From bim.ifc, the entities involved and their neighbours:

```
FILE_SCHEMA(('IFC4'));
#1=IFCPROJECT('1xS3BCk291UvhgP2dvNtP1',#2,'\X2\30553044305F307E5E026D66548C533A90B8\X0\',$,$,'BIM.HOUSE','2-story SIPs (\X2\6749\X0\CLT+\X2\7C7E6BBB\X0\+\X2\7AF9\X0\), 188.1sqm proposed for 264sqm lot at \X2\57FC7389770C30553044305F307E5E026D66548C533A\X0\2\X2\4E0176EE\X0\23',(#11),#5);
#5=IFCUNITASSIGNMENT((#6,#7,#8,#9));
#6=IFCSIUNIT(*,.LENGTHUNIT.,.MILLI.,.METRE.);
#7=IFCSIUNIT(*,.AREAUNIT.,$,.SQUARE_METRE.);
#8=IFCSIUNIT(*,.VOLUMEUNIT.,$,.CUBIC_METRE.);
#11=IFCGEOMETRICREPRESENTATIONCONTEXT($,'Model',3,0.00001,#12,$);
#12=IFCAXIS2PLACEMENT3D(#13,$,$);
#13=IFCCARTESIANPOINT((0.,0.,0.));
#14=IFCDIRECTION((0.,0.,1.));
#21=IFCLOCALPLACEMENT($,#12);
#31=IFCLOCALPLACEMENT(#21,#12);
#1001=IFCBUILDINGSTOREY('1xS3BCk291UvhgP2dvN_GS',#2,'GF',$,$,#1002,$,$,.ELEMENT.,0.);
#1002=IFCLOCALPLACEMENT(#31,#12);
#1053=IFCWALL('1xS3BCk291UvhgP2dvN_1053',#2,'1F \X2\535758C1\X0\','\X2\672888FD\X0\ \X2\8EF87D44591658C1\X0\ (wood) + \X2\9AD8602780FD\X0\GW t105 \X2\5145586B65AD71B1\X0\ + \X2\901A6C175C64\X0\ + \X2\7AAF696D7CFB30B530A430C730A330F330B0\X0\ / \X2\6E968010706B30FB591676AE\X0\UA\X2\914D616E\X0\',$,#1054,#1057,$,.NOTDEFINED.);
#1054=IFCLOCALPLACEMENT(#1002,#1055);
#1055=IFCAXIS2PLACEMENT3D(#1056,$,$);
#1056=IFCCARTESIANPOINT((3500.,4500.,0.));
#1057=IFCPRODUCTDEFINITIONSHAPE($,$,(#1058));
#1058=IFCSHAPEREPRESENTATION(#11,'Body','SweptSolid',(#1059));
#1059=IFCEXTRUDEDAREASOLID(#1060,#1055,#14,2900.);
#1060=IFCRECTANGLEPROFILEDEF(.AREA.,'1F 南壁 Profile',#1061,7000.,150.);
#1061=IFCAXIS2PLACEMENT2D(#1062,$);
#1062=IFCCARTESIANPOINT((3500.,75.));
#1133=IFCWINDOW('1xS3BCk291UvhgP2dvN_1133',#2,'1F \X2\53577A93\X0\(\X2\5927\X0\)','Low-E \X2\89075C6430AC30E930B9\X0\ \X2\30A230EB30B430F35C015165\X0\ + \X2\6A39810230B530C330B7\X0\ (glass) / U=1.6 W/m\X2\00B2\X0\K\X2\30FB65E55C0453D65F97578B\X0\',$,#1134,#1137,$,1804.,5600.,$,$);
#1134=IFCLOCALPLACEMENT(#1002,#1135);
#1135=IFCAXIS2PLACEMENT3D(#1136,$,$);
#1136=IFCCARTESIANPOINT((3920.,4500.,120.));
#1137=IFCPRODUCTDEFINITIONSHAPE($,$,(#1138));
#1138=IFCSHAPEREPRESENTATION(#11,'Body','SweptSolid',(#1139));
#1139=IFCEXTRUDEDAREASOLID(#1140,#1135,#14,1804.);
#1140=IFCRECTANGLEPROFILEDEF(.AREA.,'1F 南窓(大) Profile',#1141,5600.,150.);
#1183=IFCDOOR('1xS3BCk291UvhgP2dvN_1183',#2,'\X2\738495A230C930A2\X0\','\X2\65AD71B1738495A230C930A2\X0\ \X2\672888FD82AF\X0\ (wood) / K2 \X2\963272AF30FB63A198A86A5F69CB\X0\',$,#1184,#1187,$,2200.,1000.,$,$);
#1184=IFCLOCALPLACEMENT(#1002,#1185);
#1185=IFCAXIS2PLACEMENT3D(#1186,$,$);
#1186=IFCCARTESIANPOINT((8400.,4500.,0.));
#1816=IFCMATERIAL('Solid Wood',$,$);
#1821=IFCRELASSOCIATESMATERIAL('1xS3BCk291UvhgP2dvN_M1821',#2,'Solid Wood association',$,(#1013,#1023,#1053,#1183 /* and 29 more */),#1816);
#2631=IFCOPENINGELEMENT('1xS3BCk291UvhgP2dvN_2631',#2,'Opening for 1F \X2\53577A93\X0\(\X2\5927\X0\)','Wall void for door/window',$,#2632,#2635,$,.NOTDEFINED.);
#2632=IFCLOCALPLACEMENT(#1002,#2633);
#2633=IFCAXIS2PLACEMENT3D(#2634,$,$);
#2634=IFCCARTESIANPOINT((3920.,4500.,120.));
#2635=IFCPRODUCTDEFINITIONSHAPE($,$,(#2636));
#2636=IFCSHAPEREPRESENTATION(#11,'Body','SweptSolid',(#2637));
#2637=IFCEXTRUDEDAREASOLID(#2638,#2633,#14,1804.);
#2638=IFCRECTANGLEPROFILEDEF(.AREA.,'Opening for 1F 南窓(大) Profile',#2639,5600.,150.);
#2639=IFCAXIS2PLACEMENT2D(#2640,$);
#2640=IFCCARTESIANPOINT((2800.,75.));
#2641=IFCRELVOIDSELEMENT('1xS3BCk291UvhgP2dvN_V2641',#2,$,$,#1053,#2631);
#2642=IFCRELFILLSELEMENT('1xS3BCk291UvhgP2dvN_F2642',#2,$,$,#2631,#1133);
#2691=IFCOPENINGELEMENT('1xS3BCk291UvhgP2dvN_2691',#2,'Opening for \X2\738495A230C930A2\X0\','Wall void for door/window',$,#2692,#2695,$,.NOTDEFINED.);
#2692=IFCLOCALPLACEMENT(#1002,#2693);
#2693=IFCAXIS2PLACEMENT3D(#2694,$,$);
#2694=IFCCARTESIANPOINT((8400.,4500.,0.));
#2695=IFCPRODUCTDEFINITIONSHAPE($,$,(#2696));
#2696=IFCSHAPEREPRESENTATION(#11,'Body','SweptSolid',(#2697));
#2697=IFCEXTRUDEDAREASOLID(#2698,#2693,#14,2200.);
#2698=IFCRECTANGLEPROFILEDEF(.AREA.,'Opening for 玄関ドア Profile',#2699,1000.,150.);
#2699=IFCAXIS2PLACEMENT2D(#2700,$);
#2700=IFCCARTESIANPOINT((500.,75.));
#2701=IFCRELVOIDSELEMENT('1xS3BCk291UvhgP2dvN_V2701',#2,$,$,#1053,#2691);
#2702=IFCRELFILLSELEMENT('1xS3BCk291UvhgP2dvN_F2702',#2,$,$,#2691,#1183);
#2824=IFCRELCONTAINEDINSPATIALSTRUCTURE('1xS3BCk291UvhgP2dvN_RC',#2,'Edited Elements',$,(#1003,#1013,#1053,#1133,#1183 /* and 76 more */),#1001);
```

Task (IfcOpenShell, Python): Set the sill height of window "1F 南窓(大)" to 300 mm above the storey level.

```python
import numpy as np
import ifcopenshell
import ifcopenshell.api.geometry
import ifcopenshell.geom
import ifcopenshell.util.element
import ifcopenshell.util.placement
import ifcopenshell.util.shape
import ifcopenshell.util.unit

model = ifcopenshell.open("bim.ifc")
unit_scale = ifcopenshell.util.unit.calculate_unit_scale(model)

window = model.by_guid("1xS3BCk291UvhgP2dvN_1133")
opening = window.FillsVoids[0].RelatingOpeningElement
storey = ifcopenshell.util.element.get_container(window, ifc_class="IfcBuildingStorey")
level = ifcopenshell.util.placement.get_local_placement(storey.ObjectPlacement)[2, 3]

# The opening's origin need not be at the sill, so measure its lowest point.
shape = ifcopenshell.geom.create_shape(ifcopenshell.geom.settings(), opening)
bottom = ifcopenshell.util.shape.get_shape_bottom_elevation(shape, shape.geometry) / unit_scale
dz = level + 0.3 / unit_scale - bottom

shift = np.array([0.0, 0.0, dz])
# The window is not placed relative to its opening, so move both.
for product in (opening, window):
    matrix = ifcopenshell.util.placement.get_local_placement(product.ObjectPlacement)
    matrix[:3, 3] += shift
    ifcopenshell.api.geometry.edit_object_placement(model, product=product, matrix=matrix, is_si=False)

print(f"moved by {dz * unit_scale:+.3f} m")

model.write("bim_updated.ifc")
```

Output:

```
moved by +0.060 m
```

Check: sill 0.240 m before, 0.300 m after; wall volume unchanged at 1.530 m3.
